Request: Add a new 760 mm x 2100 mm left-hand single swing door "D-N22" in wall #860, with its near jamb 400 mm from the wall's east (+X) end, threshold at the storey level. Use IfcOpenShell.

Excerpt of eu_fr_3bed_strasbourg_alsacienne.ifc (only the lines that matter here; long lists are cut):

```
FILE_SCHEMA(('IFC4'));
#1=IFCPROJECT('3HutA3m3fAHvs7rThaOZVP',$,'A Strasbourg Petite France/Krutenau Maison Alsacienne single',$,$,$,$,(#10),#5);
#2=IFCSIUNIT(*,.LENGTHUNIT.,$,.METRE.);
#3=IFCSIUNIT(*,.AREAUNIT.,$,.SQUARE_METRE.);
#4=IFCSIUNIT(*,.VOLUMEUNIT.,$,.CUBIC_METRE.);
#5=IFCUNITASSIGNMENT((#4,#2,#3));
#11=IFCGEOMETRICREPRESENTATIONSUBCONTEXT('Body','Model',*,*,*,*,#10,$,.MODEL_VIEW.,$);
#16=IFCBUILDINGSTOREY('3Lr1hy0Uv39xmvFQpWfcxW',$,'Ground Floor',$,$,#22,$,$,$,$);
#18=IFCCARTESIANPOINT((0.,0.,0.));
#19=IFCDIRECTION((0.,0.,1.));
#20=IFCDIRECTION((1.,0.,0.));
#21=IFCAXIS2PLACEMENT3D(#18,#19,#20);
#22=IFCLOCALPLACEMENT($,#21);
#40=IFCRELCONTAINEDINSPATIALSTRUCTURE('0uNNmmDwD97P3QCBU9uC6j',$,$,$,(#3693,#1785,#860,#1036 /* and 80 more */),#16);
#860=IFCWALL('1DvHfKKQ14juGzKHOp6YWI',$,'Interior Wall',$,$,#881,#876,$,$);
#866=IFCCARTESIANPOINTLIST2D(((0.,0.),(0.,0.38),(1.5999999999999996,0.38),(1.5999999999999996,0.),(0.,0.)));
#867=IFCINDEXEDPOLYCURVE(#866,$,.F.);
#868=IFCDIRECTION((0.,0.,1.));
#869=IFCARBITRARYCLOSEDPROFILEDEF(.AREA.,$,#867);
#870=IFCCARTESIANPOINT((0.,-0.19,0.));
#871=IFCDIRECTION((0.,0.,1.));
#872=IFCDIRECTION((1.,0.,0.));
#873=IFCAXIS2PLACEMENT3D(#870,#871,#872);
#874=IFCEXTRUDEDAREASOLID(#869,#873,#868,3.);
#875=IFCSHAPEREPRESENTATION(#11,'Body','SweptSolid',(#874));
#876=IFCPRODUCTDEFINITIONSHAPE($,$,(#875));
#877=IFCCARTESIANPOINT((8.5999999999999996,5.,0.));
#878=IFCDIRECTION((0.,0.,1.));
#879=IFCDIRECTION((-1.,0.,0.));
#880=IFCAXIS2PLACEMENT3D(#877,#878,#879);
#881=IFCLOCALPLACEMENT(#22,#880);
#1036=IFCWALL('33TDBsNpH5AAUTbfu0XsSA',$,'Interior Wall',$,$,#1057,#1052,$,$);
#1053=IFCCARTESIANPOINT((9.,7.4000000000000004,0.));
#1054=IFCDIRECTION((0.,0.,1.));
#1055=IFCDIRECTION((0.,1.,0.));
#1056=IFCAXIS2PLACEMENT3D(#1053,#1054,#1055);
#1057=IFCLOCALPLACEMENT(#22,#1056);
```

```python
import numpy as np
import ifcopenshell
import ifcopenshell.api.feature
import ifcopenshell.api.geometry
import ifcopenshell.api.root
import ifcopenshell.api.spatial
import ifcopenshell.geom
import ifcopenshell.util.element
import ifcopenshell.util.placement
import ifcopenshell.util.representation
import ifcopenshell.util.shape
import ifcopenshell.util.unit

model = ifcopenshell.open("eu_fr_3bed_strasbourg_alsacienne.ifc")
unit_scale = ifcopenshell.util.unit.calculate_unit_scale(model)
settings = ifcopenshell.geom.settings()


def volume(element):
    """Net volume in cubic metres, openings subtracted."""
    shape = ifcopenshell.geom.create_shape(settings, element)
    return ifcopenshell.util.shape.get_volume(shape.geometry)


wall = model.by_guid("1DvHfKKQ14juGzKHOp6YWI")
storey = ifcopenshell.util.element.get_container(wall, ifc_class="IfcBuildingStorey")
context = ifcopenshell.util.representation.get_context(model, "Model", "Body", "MODEL_VIEW")
before = volume(wall)

width, height, from_end, sill = 0.76, 2.1, 0.4, 0.0  # metres

# The wall runs along its own X axis, and the end named is its -X end.
wall_shape = ifcopenshell.geom.create_shape(settings, wall)
x, y, z = ifcopenshell.util.shape.get_vertices(wall_shape.geometry).T
start = x.min() + from_end
face, thickness = float(y.min()), float(y.max() - y.min())
wall_matrix = ifcopenshell.util.placement.get_local_placement(wall.ObjectPlacement)
level = ifcopenshell.util.placement.get_local_placement(storey.ObjectPlacement)[2, 3]


def in_wall(x, y):
    """Placement at x, y metres in the wall's axes, at sill height."""
    matrix = wall_matrix.copy()
    matrix[:, 3] = wall_matrix @ np.array([x / unit_scale, y / unit_scale, 0.0, 1.0])
    matrix[2, 3] = level + sill / unit_scale
    return matrix


# Opening: a box that overshoots both wall faces by 50 mm.
opening = ifcopenshell.api.root.create_entity(model, ifc_class="IfcOpeningElement", predefined_type="OPENING")
box = ifcopenshell.api.geometry.add_wall_representation(
    model, context=context, length=width, height=height, thickness=thickness + 0.1
)
ifcopenshell.api.geometry.assign_representation(model, product=opening, representation=box)
ifcopenshell.api.geometry.edit_object_placement(model, product=opening, matrix=in_wall(start, face - 0.05), is_si=False)
ifcopenshell.api.feature.add_feature(model, feature=opening, element=wall)

door = ifcopenshell.api.root.create_entity(model, ifc_class="IfcDoor", name="D-N22", predefined_type="DOOR")
door.OverallWidth, door.OverallHeight = width / unit_scale, height / unit_scale
door.OperationType = "SINGLE_SWING_LEFT"
body = ifcopenshell.api.geometry.add_door_representation(
    model,
    context=context,
    overall_width=door.OverallWidth,
    overall_height=door.OverallHeight,
    operation_type="SINGLE_SWING_LEFT",
    lining_properties={"LiningDepth": thickness / unit_scale, "ThresholdDepth": thickness / unit_scale},
)
ifcopenshell.api.geometry.assign_representation(model, product=door, representation=body)
ifcopenshell.api.spatial.assign_container(model, products=[door], relating_structure=storey)
ifcopenshell.api.feature.add_filling(model, opening=opening, element=door)

# The lining spans the wall, so the door starts at the wall face.
ifcopenshell.api.geometry.edit_object_placement(model, product=door, matrix=in_wall(start, face), is_si=False)

after = volume(wall)

print(f"wall volume {before:.3f} -> {after:.3f} m3")

model.write("eu_fr_3bed_strasbourg_alsacienne_v2.ifc")
```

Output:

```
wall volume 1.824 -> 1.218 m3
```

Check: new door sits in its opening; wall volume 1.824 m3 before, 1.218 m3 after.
